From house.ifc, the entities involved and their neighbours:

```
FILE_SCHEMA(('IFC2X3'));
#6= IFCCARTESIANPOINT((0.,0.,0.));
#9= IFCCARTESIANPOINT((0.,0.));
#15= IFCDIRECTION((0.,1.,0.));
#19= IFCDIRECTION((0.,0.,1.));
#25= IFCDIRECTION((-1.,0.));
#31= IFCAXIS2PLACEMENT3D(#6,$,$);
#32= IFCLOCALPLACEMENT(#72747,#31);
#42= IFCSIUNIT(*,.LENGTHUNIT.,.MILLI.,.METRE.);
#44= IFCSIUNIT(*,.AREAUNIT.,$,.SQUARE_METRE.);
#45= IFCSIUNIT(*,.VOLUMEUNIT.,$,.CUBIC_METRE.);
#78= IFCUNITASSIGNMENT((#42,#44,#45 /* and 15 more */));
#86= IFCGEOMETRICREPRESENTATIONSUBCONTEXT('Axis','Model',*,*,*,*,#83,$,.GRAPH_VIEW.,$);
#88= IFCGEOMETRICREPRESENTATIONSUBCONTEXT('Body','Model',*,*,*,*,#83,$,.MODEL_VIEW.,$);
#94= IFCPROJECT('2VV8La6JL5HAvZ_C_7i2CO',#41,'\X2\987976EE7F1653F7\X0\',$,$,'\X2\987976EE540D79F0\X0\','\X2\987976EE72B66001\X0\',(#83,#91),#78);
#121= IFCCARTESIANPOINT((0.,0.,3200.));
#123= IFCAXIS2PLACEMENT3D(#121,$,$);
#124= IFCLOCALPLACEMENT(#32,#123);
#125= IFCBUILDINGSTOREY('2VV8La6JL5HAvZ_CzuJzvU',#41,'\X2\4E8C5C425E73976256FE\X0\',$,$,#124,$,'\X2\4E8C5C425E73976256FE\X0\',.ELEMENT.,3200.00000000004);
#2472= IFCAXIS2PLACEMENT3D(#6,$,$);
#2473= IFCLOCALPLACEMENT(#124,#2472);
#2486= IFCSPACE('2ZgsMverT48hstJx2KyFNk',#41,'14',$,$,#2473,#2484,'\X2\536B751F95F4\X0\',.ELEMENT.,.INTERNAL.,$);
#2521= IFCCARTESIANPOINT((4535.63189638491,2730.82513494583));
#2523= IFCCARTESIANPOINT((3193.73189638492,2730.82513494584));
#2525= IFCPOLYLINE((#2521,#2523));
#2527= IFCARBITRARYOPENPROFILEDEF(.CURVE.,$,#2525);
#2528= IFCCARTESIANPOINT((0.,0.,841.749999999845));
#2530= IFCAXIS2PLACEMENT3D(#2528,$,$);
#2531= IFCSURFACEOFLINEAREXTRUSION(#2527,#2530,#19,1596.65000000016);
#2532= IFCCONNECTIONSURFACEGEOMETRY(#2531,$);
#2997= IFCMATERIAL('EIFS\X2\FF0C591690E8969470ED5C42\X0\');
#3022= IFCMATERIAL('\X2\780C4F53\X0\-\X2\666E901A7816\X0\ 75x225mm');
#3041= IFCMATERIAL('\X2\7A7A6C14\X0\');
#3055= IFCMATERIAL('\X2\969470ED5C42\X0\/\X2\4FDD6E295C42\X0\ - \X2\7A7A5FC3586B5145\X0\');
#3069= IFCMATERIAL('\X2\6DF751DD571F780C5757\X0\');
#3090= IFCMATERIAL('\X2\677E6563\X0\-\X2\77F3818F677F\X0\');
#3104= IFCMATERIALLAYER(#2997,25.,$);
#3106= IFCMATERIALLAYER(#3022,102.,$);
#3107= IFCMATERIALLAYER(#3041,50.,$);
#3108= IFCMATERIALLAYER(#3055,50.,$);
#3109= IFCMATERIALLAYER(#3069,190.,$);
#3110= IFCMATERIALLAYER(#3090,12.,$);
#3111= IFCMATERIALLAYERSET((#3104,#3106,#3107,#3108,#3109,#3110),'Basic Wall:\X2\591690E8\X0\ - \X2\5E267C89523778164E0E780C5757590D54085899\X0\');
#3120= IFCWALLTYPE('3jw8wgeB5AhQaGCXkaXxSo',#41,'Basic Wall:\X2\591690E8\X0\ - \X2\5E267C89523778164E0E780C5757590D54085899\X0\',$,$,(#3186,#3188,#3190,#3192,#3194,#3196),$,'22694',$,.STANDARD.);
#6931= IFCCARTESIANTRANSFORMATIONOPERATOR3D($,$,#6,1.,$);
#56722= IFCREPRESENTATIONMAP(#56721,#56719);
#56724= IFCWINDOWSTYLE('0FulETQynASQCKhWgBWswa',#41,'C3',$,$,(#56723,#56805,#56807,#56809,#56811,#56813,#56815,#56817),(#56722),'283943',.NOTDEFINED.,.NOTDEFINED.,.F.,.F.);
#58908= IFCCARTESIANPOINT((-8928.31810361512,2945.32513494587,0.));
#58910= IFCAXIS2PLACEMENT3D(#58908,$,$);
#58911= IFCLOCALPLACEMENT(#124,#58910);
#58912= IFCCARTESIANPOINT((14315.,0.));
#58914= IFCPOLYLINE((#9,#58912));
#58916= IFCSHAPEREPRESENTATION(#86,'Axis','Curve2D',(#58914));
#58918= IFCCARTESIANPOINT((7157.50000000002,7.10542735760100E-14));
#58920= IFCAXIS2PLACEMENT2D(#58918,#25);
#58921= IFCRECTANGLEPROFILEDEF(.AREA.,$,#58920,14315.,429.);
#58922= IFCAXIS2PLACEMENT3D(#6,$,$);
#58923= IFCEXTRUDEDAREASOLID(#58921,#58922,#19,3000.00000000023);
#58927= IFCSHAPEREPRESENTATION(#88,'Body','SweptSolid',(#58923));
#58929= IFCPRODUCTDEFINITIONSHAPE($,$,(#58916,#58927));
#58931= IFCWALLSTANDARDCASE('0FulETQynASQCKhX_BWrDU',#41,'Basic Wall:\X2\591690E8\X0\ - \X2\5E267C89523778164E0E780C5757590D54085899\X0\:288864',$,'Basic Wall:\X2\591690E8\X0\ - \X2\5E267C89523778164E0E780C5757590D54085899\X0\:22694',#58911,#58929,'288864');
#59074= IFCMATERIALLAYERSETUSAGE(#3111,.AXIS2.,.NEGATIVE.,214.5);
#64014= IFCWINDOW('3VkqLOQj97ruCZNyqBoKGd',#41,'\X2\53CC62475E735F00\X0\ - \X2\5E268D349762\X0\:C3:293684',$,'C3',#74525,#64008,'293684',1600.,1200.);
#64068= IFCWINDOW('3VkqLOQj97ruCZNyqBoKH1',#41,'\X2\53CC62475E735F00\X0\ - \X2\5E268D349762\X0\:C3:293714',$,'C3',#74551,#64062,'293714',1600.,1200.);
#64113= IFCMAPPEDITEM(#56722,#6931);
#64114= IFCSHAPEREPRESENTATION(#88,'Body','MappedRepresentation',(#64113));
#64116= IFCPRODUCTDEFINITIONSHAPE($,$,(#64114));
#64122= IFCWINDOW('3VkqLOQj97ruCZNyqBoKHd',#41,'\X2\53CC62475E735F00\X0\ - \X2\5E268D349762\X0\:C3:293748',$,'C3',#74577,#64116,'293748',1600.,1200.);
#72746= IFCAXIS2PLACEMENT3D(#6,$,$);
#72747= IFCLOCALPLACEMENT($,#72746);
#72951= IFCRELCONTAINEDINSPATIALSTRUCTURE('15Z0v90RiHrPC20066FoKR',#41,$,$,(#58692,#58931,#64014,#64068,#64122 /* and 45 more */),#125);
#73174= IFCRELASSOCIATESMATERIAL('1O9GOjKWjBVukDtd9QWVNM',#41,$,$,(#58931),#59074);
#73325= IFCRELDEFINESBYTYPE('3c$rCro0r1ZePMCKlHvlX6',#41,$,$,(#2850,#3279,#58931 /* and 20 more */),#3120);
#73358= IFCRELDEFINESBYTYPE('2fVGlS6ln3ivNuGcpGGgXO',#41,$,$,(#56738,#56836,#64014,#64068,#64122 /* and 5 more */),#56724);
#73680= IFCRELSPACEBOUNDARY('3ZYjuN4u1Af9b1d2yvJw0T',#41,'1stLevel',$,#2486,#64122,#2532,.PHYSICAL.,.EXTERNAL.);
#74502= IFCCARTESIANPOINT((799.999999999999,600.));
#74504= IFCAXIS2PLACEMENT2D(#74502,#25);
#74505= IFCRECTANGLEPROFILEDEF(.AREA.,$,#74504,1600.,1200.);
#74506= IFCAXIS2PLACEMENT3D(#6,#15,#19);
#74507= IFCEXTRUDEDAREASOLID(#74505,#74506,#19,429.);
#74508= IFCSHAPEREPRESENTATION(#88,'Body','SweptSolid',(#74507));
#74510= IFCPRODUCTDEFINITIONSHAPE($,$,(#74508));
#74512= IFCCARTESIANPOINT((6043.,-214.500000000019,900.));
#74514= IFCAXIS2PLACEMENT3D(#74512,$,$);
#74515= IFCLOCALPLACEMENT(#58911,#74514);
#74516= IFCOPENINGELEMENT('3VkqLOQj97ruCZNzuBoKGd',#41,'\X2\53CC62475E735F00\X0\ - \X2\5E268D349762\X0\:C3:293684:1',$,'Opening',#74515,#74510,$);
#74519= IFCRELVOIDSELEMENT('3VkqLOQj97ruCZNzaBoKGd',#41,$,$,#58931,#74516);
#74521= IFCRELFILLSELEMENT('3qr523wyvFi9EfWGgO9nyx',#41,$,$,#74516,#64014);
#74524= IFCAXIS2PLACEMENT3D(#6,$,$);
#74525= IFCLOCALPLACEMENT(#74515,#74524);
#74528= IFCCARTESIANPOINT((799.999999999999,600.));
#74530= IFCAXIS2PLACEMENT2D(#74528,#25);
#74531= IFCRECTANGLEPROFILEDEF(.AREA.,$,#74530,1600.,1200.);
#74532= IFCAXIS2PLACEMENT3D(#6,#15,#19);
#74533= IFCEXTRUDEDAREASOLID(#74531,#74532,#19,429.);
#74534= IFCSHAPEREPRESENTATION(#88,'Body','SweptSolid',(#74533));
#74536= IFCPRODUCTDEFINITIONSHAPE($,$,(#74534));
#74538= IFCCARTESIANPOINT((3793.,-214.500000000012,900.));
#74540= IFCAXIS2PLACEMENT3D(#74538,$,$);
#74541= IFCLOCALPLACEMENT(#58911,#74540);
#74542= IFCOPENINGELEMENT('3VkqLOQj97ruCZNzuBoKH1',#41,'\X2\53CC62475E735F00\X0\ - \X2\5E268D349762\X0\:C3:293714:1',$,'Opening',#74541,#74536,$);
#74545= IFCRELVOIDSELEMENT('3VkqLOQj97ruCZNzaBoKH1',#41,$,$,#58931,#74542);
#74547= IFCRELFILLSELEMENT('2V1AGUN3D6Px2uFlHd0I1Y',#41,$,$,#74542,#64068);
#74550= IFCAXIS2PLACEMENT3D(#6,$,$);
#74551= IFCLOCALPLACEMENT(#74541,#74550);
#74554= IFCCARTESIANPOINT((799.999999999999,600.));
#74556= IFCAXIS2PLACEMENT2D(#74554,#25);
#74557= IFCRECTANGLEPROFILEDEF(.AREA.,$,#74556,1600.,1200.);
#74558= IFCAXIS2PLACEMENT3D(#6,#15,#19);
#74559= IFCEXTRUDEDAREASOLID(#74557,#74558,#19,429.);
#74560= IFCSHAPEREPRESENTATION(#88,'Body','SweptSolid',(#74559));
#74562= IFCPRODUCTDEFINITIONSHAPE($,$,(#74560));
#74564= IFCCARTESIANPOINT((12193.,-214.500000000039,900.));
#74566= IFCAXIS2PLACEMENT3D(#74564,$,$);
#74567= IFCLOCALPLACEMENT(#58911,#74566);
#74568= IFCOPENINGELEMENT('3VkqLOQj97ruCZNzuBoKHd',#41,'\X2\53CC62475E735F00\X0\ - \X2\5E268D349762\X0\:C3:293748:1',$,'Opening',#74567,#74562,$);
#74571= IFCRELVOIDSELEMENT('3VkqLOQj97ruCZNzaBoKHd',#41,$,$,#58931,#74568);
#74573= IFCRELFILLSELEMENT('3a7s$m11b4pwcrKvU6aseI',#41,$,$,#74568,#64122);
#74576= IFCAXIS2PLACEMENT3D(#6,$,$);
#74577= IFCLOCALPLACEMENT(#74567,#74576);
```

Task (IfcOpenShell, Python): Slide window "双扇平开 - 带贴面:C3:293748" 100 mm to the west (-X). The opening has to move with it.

```python
import numpy as np
import ifcopenshell
import ifcopenshell.api.geometry
import ifcopenshell.util.placement

model = ifcopenshell.open("house.ifc")

window = model.by_guid("3VkqLOQj97ruCZNyqBoKHd")
opening = window.FillsVoids[0].RelatingOpeningElement
wall = opening.VoidsElements[0].RelatingBuildingElement

wall_matrix = ifcopenshell.util.placement.get_local_placement(wall.ObjectPlacement)
shift = wall_matrix[:3, 0] * -100.0
before = ifcopenshell.util.placement.get_local_placement(window.ObjectPlacement)[:3, 3].copy()

# The window is placed relative to its opening, so it follows when the opening moves.
matrix = ifcopenshell.util.placement.get_local_placement(opening.ObjectPlacement)
matrix[:3, 3] += shift
ifcopenshell.api.geometry.edit_object_placement(
    model, product=opening, matrix=matrix, is_si=False, should_transform_children=True
)

# Space boundary surfaces are stored in each space's coordinates; move them too.
for rel in window.ProvidesBoundaries:
    if not rel.ConnectionGeometry:
        continue
    surface = rel.ConnectionGeometry.SurfaceOnRelatingElement
    space_matrix = ifcopenshell.util.placement.get_local_placement(rel.RelatingSpace.ObjectPlacement)
    point = np.array(surface.Position.Location.Coordinates) + space_matrix[:3, :3].T @ shift
    surface.Position = model.createIfcAxis2Placement3D(
        model.createIfcCartesianPoint(point.tolist()), surface.Position.Axis, surface.Position.RefDirection
    )

after = ifcopenshell.util.placement.get_local_placement(window.ObjectPlacement)[:3, 3]
print("window moved by", (after - before).round(3) + 0.0)

model.write("house-out.ifc")
```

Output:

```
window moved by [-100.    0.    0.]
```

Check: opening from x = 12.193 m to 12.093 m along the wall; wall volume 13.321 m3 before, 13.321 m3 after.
